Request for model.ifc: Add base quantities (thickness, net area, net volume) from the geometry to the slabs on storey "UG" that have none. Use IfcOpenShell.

First a look at what the model holds.

```python
import ifcopenshell
import ifcopenshell.util.element
import ifcopenshell.util.unit

model = ifcopenshell.open("model.ifc")
print(model.schema)
for unit_type in ("LENGTHUNIT", "AREAUNIT", "VOLUMEUNIT"):
    print(unit_type, ifcopenshell.util.unit.calculate_unit_scale(model, unit_type))
storey = next(s for s in model.by_type("IfcBuildingStorey") if s.Name == "UG")
slabs = [e for e in ifcopenshell.util.element.get_decomposition(storey) if e.is_a("IfcSlab")]
for e in sorted(slabs, key=lambda e: e.id()):
    print(e.id(), e.is_a(), e.Name, list(ifcopenshell.util.element.get_psets(e, qtos_only=True)), sep=" | ")
```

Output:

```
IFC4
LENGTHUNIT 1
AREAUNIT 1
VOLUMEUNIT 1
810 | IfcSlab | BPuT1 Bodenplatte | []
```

```python
import ifcopenshell
import ifcopenshell.api.pset
import ifcopenshell.geom
import ifcopenshell.util.element
import ifcopenshell.util.shape
import ifcopenshell.util.unit

model = ifcopenshell.open("model.ifc")
unit_scale = ifcopenshell.util.unit.calculate_unit_scale(model)
area_scale = ifcopenshell.util.unit.calculate_unit_scale(model, "AREAUNIT")
volume_scale = ifcopenshell.util.unit.calculate_unit_scale(model, "VOLUMEUNIT")
settings = ifcopenshell.geom.settings()

storey = next(s for s in model.by_type("IfcBuildingStorey") if s.Name == "UG")
slabs = [e for e in ifcopenshell.util.element.get_decomposition(storey) if e.is_a("IfcSlab")]

for e in sorted(slabs, key=lambda e: e.id()):
    if ifcopenshell.util.element.get_psets(e, qtos_only=True, should_inherit=False):
        continue
    # Geometry comes back in metres, in the element's own axes.
    shape = ifcopenshell.geom.create_shape(settings, e)
    values = {
        "Width": ifcopenshell.util.shape.get_z(shape.geometry) / unit_scale,
        "NetArea": ifcopenshell.util.shape.get_footprint_area(shape.geometry) / area_scale,
        "NetVolume": ifcopenshell.util.shape.get_volume(shape.geometry) / volume_scale,
    }
    qto = ifcopenshell.api.pset.add_qto(model, product=e, name="Qto_SlabBaseQuantities")
    ifcopenshell.api.pset.edit_qto(model, qto=qto, properties=values)
    print(e.id(), {k: round(v, 3) for k, v in values.items()})

model.write("model-out.ifc")
```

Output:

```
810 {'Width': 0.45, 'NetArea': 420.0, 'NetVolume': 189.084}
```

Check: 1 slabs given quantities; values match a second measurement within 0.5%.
